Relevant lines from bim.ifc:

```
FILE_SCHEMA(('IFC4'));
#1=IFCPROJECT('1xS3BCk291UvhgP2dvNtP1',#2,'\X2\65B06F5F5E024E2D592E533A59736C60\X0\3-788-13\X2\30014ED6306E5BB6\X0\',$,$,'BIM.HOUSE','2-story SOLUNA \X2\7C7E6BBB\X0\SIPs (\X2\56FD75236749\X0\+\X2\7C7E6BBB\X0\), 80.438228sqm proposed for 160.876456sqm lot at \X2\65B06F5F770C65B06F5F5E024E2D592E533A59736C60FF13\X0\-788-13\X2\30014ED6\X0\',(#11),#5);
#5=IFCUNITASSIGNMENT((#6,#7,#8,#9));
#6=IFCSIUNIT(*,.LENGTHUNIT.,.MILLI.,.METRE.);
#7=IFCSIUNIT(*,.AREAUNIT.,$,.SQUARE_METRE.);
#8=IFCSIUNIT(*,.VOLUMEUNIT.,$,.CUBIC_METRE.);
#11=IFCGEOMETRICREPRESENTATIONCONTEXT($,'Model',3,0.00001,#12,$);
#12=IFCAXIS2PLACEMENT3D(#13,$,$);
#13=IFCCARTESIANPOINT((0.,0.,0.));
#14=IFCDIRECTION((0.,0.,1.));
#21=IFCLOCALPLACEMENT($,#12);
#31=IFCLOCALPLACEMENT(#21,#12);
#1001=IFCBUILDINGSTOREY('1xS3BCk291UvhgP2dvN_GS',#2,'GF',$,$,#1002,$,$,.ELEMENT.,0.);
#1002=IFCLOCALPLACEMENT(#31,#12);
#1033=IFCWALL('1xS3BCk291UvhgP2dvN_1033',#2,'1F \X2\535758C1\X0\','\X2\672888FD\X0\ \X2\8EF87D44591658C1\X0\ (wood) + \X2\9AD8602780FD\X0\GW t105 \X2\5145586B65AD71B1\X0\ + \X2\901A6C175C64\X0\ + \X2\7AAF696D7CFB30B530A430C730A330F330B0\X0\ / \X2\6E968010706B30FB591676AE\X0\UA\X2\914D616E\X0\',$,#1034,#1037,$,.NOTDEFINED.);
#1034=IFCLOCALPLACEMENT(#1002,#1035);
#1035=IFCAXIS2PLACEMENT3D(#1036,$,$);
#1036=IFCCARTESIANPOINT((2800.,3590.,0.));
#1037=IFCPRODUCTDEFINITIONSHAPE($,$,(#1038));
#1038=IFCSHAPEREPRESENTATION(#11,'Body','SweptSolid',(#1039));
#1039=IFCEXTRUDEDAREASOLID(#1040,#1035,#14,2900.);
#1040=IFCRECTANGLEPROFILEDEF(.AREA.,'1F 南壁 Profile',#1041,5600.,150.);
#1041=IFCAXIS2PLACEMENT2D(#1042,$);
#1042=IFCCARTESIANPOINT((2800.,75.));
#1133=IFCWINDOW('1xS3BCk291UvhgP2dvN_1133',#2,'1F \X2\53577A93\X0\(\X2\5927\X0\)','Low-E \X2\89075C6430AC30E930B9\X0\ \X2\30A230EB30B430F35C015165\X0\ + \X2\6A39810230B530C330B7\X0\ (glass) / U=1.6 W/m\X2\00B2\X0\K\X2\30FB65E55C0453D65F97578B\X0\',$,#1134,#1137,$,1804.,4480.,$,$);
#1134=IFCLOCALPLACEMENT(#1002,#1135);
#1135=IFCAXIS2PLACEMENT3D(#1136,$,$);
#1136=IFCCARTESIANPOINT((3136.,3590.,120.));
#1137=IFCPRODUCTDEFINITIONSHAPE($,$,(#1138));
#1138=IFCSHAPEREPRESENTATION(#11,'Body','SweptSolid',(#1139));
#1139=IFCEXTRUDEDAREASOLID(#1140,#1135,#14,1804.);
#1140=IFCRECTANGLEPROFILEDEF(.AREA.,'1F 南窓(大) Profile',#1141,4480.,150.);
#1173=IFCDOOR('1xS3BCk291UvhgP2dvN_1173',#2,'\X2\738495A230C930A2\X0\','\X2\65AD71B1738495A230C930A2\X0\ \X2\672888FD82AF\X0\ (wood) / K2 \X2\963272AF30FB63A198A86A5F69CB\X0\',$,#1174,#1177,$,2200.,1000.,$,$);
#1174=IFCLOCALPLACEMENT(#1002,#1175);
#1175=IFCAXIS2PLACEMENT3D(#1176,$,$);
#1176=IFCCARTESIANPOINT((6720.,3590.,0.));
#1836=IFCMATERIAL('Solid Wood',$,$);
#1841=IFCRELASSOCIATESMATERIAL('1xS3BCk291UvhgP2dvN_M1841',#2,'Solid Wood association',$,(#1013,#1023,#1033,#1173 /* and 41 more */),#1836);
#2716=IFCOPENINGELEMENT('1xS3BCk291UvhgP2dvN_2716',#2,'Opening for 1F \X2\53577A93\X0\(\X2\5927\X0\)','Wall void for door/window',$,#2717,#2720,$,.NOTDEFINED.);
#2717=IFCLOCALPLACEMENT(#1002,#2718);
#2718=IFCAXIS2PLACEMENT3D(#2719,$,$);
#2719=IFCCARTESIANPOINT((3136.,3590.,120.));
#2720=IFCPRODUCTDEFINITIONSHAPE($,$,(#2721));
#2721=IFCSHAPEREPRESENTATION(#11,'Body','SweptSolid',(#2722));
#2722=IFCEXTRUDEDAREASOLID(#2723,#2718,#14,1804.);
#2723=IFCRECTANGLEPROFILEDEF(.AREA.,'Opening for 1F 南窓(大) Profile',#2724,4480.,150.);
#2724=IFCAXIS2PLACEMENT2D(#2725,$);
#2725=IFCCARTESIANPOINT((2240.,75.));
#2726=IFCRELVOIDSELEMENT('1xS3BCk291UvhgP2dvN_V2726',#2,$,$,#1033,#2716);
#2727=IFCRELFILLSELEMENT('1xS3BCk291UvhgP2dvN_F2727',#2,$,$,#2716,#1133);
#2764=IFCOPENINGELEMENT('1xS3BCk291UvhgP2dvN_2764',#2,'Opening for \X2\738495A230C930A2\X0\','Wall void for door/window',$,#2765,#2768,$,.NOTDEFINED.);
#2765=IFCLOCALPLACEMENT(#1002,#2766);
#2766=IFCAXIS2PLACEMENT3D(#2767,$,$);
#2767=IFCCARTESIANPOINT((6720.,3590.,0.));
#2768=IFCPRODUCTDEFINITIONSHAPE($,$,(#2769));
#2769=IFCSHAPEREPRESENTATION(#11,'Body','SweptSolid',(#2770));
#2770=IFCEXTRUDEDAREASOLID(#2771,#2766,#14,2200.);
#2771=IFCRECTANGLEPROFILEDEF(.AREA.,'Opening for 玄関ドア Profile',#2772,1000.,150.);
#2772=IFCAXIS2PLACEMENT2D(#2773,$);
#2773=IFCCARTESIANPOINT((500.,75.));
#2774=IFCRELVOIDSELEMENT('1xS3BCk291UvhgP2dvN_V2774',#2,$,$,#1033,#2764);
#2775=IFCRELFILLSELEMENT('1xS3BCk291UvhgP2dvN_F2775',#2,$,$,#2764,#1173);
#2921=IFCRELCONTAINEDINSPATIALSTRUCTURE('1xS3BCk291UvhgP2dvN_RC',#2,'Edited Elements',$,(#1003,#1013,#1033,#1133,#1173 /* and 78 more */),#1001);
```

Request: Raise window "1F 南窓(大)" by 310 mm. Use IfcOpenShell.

```python
import numpy as np
import ifcopenshell
import ifcopenshell.api.geometry
import ifcopenshell.util.placement
import ifcopenshell.util.unit

model = ifcopenshell.open("bim.ifc")
unit_scale = ifcopenshell.util.unit.calculate_unit_scale(model)

window = model.by_guid("1xS3BCk291UvhgP2dvN_1133")
opening = window.FillsVoids[0].RelatingOpeningElement
dz = 0.31 / unit_scale

shift = np.array([0.0, 0.0, dz])
# The window is not placed relative to its opening, so move both.
for product in (opening, window):
    matrix = ifcopenshell.util.placement.get_local_placement(product.ObjectPlacement)
    matrix[:3, 3] += shift
    ifcopenshell.api.geometry.edit_object_placement(model, product=product, matrix=matrix, is_si=False)

print(f"moved by {dz * unit_scale:+.3f} m")

model.write("bim_edited.ifc")
```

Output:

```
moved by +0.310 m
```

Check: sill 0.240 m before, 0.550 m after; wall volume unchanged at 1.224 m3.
